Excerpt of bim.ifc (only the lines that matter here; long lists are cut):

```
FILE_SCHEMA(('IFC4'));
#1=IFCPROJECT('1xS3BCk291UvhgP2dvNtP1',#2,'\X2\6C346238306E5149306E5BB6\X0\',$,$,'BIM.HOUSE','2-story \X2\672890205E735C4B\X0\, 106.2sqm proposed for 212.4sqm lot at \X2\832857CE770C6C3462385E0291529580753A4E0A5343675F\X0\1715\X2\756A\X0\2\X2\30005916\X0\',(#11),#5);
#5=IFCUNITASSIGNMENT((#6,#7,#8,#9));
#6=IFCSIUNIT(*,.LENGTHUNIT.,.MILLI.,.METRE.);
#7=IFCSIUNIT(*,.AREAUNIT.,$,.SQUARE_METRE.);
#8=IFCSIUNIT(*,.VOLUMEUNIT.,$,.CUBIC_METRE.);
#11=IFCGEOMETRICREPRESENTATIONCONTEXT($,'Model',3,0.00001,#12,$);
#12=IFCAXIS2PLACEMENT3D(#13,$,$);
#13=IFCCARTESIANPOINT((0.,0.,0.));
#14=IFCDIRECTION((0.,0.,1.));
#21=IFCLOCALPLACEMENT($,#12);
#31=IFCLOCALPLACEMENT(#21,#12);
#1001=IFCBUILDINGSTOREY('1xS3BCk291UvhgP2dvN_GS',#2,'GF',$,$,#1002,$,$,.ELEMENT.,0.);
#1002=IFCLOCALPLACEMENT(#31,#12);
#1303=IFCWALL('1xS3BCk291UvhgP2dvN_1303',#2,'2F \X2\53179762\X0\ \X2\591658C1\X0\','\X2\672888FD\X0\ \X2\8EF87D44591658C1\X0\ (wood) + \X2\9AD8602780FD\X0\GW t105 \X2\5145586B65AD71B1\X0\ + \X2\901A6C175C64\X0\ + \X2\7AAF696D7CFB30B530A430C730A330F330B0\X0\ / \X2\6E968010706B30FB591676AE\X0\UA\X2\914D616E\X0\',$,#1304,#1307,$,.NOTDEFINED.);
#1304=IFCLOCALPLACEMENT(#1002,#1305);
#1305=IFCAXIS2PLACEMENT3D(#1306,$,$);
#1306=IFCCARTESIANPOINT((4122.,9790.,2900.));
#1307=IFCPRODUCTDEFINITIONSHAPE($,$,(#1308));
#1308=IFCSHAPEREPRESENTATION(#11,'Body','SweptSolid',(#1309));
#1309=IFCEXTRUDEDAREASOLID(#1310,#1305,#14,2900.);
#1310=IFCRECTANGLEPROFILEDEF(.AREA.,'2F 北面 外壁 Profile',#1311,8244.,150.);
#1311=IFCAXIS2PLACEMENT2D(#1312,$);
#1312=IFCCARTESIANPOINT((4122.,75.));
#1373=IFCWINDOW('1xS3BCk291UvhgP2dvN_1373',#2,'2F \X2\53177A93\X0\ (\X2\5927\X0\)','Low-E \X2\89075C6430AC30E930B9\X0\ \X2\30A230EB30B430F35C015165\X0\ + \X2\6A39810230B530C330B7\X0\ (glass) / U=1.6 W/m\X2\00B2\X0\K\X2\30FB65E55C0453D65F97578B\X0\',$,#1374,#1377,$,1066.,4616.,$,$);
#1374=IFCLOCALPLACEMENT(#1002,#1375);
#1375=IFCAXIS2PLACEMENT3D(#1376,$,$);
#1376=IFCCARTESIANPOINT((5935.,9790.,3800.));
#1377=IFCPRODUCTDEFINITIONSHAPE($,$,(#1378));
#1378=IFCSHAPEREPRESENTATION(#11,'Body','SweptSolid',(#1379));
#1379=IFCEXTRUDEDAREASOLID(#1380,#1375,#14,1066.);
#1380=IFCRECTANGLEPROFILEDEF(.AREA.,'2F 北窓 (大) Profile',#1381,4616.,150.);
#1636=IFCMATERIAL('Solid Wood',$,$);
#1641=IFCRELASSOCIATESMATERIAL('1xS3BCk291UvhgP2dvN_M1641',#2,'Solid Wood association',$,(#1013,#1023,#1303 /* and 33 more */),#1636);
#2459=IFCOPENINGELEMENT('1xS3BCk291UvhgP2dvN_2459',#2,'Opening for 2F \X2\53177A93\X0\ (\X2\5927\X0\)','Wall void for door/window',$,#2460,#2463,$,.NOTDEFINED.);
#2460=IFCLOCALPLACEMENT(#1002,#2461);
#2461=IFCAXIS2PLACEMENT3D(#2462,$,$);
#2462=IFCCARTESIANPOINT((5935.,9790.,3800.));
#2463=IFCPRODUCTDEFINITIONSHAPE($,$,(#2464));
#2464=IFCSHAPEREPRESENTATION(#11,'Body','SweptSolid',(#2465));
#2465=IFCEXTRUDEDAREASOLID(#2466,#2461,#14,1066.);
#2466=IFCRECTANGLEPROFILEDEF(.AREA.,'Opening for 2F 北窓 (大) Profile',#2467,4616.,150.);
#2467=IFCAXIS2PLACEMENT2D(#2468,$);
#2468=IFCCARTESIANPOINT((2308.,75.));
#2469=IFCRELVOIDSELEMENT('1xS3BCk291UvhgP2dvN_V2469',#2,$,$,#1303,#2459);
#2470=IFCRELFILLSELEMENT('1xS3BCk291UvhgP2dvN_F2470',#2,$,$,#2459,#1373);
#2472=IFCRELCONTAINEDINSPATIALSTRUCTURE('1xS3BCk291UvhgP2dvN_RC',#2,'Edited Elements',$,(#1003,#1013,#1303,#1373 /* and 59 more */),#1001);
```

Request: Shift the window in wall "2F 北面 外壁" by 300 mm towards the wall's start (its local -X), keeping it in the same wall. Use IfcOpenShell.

```python
import ifcopenshell
import ifcopenshell.api.geometry
import ifcopenshell.util.placement
import ifcopenshell.util.unit

model = ifcopenshell.open("bim.ifc")
unit_scale = ifcopenshell.util.unit.calculate_unit_scale(model)

window = model.by_id(1373)
opening = window.FillsVoids[0].RelatingOpeningElement
wall = opening.VoidsElements[0].RelatingBuildingElement

wall_matrix = ifcopenshell.util.placement.get_local_placement(wall.ObjectPlacement)
shift = wall_matrix[:3, 0] * -0.3 / unit_scale
before = ifcopenshell.util.placement.get_local_placement(window.ObjectPlacement)[:3, 3].copy()

# The window is not placed relative to its opening, so move both.
for product in (opening, window):
    matrix = ifcopenshell.util.placement.get_local_placement(product.ObjectPlacement)
    matrix[:3, 3] += shift
    ifcopenshell.api.geometry.edit_object_placement(model, product=product, matrix=matrix, is_si=False)

after = ifcopenshell.util.placement.get_local_placement(window.ObjectPlacement)[:3, 3]
print("window moved by", (after - before).round(3) + 0.0)

model.write("bim_edited.ifc")
```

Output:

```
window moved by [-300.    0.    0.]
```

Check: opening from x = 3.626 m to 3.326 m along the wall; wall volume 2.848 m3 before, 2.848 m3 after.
